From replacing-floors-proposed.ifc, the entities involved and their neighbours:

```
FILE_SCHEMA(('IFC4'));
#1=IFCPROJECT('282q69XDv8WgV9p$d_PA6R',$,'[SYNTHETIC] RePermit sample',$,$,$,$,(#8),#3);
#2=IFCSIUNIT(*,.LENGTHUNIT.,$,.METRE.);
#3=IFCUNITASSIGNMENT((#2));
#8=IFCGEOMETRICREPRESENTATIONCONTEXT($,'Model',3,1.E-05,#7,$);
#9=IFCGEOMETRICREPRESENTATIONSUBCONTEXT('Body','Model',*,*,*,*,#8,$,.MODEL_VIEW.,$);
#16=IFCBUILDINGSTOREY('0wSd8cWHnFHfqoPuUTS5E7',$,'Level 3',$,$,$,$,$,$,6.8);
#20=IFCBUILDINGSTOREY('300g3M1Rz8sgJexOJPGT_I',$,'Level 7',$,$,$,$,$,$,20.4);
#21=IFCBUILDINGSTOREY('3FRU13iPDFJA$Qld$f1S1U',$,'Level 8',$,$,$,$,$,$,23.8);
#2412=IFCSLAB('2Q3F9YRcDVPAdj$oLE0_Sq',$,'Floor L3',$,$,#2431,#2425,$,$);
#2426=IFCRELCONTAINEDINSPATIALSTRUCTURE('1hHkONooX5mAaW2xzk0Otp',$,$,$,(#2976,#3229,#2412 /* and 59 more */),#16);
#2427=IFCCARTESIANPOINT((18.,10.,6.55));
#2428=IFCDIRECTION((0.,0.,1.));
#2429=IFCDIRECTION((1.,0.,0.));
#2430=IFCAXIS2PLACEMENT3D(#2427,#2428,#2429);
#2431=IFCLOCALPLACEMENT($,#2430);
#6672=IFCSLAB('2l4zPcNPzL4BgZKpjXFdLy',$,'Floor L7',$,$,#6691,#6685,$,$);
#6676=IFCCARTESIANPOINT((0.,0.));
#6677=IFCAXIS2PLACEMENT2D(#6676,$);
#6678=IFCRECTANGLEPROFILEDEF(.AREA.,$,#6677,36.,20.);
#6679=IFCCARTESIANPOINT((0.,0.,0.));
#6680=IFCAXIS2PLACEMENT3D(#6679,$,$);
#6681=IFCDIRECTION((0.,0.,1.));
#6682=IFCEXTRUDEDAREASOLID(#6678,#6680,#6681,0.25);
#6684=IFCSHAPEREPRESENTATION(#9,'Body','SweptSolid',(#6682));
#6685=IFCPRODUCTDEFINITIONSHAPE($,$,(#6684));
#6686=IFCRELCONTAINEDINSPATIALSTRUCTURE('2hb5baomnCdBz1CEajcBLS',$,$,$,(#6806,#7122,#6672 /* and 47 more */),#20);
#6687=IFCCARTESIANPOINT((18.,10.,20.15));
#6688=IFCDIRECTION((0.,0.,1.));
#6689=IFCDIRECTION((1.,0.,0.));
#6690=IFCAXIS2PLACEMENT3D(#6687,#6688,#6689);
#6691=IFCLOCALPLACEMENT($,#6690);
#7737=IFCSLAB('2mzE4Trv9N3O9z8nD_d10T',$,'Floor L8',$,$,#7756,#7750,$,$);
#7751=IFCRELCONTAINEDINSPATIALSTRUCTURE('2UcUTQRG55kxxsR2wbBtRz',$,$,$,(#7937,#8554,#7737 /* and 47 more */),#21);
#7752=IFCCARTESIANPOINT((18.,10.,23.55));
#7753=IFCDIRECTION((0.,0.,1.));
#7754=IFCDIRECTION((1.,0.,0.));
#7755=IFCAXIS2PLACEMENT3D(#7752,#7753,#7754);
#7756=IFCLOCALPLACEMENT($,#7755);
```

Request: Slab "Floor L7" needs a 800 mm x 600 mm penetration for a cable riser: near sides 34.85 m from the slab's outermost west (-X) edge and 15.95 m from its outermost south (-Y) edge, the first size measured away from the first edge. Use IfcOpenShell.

```python
import numpy as np
import ifcopenshell
import ifcopenshell.api.feature
import ifcopenshell.api.geometry
import ifcopenshell.api.root
import ifcopenshell.geom
import ifcopenshell.util.placement
import ifcopenshell.util.representation
import ifcopenshell.util.shape
import ifcopenshell.util.unit

model = ifcopenshell.open("replacing-floors-proposed.ifc")
unit_scale = ifcopenshell.util.unit.calculate_unit_scale(model)
settings = ifcopenshell.geom.settings()


def volume(element):
    """Net volume in cubic metres, openings subtracted."""
    shape = ifcopenshell.geom.create_shape(settings, element)
    return ifcopenshell.util.shape.get_volume(shape.geometry)


slab = model.by_guid("2l4zPcNPzL4BgZKpjXFdLy")
before = volume(slab)

# Extent in the slab's own axes, in metres. The edges named are its -X and -Y sides.
slab_shape = ifcopenshell.geom.create_shape(settings, slab)
vertices = ifcopenshell.util.shape.get_vertices(slab_shape.geometry)
x_min, y_min, bottom = vertices.min(axis=0)
top = vertices[:, 2].max()

opening = ifcopenshell.api.root.create_entity(model, ifc_class="IfcOpeningElement", name="Cable riser opening", predefined_type="OPENING")
context = ifcopenshell.util.representation.get_context(model, "Model", "Body", "MODEL_VIEW")
width, depth = 0.8, 0.6
outline = [(0.0, 0.0), (width, 0.0), (width, depth), (0.0, depth), (0.0, 0.0)]
# Overshoot both faces by 50 mm so the cut is clean.
shape = ifcopenshell.api.geometry.add_slab_representation(
    model, context=context, depth=top - bottom + 0.1, polyline=outline
)
ifcopenshell.api.geometry.assign_representation(model, product=opening, representation=shape)

matrix = ifcopenshell.util.placement.get_local_placement(slab.ObjectPlacement)
matrix[:, 3] = matrix @ np.append(np.array([x_min + 34.85, y_min + 15.95, bottom - 0.05]) / unit_scale, 1.0)
ifcopenshell.api.geometry.edit_object_placement(model, product=opening, matrix=matrix, is_si=False)
ifcopenshell.api.feature.add_feature(model, feature=opening, element=slab)

after = volume(slab)

print(f"slab volume {before:.3f} -> {after:.3f} m3")

model.write("replacing-floors-proposed_updated.ifc")
```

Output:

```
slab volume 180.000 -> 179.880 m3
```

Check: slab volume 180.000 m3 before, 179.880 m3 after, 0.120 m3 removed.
